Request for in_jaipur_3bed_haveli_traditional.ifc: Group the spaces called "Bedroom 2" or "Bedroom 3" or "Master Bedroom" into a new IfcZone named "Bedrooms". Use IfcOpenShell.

First a look at what the model holds.

```python
import ifcopenshell

model = ifcopenshell.open("in_jaipur_3bed_haveli_traditional.ifc")
print(model.schema)
seen = {}
for space in model.by_type("IfcSpace"):
    seen[space.LongName] = seen.get(space.LongName, 0) + 1
for name, count in sorted(seen.items(), key=str):
    print(count, "x", name)
print("zones:", [z.Name for z in model.by_type("IfcZone")][:20])
```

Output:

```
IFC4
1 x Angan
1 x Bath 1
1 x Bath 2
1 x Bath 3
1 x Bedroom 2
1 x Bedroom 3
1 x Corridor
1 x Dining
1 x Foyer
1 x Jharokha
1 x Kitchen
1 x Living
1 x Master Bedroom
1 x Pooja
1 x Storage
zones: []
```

```python
import ifcopenshell
import ifcopenshell.api.group
import ifcopenshell.api.root

model = ifcopenshell.open("in_jaipur_3bed_haveli_traditional.ifc")

names = {"Bedroom 2", "Bedroom 3", "Master Bedroom"}
spaces = [s for s in model.by_type("IfcSpace") if s.LongName in names]

zone = ifcopenshell.api.root.create_entity(model, ifc_class="IfcZone", name="Bedrooms")
ifcopenshell.api.group.assign_group(model, products=spaces, group=zone)
print(len(spaces), "spaces in", zone.Name)

model.write("in_jaipur_3bed_haveli_traditional_updated.ifc")
```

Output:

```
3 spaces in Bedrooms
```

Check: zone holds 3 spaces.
